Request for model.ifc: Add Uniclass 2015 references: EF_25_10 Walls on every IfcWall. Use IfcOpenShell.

First a look at what the model holds.

```python
import ifcopenshell

model = ifcopenshell.open("model.ifc")
print(model.schema)
print("classifications:", [c.Name for c in model.by_type("IfcClassification")])
for ifc_class in ("IfcDoor", "IfcRoof", "IfcStair", "IfcWall", "IfcWindow"):
    print(ifc_class, len(model.by_type(ifc_class)))
```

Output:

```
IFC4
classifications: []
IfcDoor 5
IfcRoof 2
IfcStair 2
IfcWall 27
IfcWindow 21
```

```python
import ifcopenshell
import ifcopenshell.api.classification

model = ifcopenshell.open("model.ifc")

system = ifcopenshell.api.classification.add_classification(model, classification="Uniclass 2015")

codes = {
    "IfcWall": ("EF_25_10", "Walls"),
}
for ifc_class, (code, name) in codes.items():
    products = model.by_type(ifc_class)
    ifcopenshell.api.classification.add_reference(
        model, products=products, classification=system, identification=code, name=name
    )
    print(code, len(products))

model.write("model_rev.ifc")
```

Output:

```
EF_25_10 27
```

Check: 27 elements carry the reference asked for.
